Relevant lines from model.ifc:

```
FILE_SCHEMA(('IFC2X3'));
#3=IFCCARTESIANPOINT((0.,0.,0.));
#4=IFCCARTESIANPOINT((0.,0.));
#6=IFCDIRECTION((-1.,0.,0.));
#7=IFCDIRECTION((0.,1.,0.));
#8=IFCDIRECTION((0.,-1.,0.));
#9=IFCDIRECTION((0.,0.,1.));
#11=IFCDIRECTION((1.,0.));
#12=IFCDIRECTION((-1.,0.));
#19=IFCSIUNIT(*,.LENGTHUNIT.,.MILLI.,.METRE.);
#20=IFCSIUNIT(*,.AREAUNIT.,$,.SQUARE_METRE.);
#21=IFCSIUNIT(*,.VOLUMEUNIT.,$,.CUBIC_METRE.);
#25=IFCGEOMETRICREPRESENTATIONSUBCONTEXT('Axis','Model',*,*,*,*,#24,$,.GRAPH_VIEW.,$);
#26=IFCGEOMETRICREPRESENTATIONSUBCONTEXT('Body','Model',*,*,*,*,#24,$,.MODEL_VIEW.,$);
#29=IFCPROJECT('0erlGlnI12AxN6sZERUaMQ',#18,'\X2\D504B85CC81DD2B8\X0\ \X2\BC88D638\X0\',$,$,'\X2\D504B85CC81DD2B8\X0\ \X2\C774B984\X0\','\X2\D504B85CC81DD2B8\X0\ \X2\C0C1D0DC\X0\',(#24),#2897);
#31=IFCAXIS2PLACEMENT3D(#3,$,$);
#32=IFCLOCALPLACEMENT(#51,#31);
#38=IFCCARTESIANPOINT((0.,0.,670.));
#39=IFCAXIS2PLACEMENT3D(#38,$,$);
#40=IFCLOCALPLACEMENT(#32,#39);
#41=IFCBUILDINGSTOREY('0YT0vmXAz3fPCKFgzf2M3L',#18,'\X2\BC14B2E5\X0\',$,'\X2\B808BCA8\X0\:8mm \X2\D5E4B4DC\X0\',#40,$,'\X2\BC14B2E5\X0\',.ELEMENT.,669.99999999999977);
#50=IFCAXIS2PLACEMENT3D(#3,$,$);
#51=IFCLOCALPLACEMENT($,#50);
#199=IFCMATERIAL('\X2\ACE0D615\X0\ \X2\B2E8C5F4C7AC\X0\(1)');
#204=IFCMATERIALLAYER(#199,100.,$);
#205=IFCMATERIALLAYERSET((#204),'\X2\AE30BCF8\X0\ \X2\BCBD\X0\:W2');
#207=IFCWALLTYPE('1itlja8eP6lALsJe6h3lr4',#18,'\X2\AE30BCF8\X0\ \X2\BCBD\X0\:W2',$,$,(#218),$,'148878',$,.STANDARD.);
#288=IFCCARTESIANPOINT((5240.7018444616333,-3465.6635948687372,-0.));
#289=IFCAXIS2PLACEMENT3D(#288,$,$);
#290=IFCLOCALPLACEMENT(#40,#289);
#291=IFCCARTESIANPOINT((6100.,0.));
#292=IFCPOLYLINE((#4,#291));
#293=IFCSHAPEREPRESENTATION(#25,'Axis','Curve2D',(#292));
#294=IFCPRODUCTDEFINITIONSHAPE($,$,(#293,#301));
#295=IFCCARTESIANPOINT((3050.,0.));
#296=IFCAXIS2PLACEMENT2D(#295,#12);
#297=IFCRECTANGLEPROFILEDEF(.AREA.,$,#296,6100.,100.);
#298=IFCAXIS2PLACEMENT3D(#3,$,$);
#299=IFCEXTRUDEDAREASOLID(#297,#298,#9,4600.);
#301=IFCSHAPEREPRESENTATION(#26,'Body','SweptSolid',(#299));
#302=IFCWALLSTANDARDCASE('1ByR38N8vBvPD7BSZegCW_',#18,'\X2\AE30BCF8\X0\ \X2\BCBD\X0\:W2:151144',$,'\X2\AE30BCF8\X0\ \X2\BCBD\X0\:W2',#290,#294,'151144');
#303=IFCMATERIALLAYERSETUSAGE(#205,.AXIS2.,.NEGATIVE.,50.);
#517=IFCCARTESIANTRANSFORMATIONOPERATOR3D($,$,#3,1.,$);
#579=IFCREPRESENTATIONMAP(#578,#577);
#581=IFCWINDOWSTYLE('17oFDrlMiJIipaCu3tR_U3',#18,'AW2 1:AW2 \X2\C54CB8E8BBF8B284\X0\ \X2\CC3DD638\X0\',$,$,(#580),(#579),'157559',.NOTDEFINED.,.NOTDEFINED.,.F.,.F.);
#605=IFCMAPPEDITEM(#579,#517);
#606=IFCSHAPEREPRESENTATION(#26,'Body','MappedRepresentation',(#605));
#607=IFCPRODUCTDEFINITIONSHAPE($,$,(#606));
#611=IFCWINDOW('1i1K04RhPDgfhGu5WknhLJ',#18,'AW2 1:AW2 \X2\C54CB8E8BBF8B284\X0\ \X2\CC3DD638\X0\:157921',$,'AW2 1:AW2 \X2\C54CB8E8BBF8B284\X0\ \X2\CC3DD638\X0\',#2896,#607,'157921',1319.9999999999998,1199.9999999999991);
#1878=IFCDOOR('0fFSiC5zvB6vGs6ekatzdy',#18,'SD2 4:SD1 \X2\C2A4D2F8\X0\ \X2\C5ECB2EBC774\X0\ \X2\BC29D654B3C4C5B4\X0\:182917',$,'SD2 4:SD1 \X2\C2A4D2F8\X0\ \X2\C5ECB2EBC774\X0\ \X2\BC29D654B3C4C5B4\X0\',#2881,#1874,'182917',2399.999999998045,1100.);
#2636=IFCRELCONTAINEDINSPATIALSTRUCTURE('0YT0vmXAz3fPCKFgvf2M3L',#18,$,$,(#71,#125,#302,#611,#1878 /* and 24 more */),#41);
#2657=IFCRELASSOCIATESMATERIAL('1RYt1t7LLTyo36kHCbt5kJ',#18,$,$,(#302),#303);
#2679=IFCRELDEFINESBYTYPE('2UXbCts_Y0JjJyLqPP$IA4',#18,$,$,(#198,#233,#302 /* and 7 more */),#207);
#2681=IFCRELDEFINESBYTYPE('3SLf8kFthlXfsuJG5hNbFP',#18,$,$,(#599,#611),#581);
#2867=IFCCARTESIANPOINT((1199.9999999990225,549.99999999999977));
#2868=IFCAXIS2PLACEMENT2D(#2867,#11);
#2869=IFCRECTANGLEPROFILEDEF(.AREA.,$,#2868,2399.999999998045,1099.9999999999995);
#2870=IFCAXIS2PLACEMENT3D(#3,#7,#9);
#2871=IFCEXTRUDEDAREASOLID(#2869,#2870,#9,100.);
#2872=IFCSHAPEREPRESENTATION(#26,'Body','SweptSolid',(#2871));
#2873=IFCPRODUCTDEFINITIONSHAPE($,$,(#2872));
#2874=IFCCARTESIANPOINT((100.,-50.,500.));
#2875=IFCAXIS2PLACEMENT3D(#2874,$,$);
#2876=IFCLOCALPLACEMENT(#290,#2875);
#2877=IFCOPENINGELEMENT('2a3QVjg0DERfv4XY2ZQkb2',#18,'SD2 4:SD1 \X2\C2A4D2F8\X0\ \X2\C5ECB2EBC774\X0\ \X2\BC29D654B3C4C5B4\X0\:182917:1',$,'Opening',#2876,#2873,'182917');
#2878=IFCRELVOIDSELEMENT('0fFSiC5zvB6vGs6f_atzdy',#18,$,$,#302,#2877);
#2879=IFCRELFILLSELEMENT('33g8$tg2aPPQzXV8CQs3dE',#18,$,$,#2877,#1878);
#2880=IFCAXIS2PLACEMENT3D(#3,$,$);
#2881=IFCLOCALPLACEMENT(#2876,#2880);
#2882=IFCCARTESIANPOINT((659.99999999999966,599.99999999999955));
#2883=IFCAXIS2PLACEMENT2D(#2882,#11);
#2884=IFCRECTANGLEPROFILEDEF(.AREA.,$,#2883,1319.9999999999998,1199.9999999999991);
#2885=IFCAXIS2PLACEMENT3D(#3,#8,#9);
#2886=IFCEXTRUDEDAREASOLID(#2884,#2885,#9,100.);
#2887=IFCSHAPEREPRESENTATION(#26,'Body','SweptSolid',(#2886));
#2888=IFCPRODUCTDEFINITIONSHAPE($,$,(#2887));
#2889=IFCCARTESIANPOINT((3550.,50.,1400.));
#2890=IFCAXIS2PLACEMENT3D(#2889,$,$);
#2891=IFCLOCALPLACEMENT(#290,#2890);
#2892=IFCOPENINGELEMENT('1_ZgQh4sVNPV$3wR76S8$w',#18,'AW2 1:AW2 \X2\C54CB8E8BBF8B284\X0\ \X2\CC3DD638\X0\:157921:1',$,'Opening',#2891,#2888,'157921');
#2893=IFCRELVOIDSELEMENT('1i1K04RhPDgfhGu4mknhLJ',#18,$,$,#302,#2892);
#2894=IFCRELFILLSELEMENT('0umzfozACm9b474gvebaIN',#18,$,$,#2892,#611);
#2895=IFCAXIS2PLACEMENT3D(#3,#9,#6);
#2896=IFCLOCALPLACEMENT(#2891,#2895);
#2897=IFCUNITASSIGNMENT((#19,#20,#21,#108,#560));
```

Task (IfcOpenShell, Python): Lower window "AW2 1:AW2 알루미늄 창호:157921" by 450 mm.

```python
import numpy as np
import ifcopenshell
import ifcopenshell.api.geometry
import ifcopenshell.util.placement
import ifcopenshell.util.unit

model = ifcopenshell.open("model.ifc")
unit_scale = ifcopenshell.util.unit.calculate_unit_scale(model)

window = model.by_guid("1i1K04RhPDgfhGu5WknhLJ")
opening = window.FillsVoids[0].RelatingOpeningElement
dz = -0.45 / unit_scale

shift = np.array([0.0, 0.0, dz])
# The window is placed relative to its opening, so it follows when the opening moves.
matrix = ifcopenshell.util.placement.get_local_placement(opening.ObjectPlacement)
matrix[:3, 3] += shift
ifcopenshell.api.geometry.edit_object_placement(
    model, product=opening, matrix=matrix, is_si=False, should_transform_children=True
)

print(f"moved by {dz * unit_scale:+.3f} m")

model.write("model-out.ifc")
```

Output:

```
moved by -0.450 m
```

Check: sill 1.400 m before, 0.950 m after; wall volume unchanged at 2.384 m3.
